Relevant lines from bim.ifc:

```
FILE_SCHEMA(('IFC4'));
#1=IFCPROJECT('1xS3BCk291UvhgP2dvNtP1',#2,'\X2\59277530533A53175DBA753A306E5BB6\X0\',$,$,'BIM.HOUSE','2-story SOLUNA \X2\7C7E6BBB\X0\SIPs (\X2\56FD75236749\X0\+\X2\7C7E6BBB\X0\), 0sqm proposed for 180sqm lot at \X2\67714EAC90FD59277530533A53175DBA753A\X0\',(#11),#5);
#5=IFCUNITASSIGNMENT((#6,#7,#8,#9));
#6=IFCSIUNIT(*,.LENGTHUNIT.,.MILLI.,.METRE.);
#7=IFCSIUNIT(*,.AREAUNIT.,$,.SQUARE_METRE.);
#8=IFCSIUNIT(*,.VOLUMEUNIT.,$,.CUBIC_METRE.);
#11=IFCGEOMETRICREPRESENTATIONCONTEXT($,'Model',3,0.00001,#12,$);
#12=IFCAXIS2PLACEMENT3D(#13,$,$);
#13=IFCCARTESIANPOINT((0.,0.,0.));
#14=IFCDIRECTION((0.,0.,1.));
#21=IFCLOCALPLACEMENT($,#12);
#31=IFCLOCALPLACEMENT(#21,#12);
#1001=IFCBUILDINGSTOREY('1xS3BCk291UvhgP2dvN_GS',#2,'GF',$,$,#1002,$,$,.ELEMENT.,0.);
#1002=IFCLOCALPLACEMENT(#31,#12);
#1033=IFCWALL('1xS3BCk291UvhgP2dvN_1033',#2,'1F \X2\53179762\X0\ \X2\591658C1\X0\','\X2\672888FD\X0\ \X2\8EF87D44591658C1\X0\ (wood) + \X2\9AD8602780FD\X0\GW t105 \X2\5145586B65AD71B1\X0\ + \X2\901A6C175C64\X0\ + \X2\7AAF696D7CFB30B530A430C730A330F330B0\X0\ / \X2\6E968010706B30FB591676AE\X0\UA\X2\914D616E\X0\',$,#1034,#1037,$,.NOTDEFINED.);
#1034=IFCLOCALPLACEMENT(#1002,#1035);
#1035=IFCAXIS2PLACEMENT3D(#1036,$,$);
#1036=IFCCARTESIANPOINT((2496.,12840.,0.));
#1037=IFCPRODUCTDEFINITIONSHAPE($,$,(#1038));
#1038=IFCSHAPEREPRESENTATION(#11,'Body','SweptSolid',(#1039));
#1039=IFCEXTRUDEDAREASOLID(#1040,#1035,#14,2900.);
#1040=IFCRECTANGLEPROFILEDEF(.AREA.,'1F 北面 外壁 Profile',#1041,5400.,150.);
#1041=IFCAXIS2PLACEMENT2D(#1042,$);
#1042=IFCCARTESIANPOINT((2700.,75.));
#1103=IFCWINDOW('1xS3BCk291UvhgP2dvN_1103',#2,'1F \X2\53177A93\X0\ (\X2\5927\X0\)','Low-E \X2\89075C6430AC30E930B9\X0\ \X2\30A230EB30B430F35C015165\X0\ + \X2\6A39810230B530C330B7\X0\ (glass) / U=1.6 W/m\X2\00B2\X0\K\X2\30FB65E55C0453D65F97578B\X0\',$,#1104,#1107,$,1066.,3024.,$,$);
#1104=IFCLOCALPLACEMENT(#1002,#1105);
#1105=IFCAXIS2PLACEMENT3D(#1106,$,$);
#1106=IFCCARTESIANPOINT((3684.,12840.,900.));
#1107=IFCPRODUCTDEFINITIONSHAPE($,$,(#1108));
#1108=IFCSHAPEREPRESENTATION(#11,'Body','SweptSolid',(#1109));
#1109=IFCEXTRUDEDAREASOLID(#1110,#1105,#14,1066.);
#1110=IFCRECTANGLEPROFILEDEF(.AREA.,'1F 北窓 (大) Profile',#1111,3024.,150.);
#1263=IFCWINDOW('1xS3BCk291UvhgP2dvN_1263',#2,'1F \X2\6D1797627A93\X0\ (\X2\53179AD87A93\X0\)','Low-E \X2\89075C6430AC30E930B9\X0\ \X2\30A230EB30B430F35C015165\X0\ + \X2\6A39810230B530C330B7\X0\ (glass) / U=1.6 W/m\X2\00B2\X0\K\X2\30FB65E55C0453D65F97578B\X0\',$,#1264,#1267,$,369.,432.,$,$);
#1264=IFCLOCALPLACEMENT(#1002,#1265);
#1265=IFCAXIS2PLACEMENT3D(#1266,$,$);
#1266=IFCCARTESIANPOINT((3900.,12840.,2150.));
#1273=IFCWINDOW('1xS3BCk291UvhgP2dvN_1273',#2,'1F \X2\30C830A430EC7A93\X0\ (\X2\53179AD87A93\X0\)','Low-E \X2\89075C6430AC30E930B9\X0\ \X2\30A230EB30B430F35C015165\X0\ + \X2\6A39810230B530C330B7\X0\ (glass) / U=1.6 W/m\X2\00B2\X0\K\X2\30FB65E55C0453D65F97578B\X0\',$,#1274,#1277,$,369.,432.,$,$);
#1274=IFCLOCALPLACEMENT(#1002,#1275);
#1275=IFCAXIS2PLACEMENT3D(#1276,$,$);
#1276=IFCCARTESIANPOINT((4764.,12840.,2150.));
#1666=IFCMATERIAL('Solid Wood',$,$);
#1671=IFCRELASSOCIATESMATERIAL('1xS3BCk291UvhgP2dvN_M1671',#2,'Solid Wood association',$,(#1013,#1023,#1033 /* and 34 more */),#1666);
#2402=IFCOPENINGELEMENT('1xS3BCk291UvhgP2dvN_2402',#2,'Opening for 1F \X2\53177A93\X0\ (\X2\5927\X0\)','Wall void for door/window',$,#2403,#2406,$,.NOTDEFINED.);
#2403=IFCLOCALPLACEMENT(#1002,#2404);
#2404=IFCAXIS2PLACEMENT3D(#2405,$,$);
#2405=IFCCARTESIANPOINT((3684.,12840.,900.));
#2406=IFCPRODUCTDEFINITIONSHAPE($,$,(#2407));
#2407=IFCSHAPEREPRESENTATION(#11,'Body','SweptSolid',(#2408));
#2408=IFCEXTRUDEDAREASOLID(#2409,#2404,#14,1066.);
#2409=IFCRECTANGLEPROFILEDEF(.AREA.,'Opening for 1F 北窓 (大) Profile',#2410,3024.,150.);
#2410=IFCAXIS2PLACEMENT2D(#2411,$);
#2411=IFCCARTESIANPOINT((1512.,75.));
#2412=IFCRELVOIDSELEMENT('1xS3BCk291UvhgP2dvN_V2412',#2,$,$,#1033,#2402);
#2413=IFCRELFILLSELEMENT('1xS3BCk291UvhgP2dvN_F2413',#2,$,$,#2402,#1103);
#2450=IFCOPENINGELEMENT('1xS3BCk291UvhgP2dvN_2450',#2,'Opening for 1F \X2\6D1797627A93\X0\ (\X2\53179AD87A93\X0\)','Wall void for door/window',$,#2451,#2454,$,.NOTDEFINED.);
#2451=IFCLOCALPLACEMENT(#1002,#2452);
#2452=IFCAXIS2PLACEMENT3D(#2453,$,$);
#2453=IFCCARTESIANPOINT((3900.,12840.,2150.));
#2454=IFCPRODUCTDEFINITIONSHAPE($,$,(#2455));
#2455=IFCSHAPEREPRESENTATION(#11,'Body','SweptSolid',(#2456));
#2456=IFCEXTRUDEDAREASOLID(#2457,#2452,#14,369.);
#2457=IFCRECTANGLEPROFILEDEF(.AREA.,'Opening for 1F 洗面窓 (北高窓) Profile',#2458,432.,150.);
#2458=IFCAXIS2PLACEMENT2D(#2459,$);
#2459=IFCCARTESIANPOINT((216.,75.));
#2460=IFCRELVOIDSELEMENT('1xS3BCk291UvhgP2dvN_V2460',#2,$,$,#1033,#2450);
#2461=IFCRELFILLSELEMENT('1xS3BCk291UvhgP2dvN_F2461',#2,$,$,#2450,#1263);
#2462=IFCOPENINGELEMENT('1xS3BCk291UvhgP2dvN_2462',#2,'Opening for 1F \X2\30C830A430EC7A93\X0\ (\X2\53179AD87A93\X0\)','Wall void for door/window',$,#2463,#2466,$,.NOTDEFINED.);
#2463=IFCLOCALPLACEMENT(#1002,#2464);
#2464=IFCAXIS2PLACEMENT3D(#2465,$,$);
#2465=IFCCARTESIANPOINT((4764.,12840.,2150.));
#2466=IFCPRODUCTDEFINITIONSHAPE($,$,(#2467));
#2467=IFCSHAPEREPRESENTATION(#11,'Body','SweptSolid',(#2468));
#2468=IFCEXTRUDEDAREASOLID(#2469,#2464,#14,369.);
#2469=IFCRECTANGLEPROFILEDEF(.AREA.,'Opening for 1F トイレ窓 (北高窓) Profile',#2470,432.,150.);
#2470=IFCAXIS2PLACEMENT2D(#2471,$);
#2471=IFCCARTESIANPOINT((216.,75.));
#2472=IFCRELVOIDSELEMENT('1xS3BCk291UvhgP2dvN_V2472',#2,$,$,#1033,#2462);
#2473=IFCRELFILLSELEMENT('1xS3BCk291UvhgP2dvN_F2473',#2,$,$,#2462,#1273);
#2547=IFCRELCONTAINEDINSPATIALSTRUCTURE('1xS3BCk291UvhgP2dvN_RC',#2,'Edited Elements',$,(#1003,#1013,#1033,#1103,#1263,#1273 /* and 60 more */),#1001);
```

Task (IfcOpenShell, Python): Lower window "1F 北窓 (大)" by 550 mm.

```python
import numpy as np
import ifcopenshell
import ifcopenshell.api.geometry
import ifcopenshell.util.placement
import ifcopenshell.util.unit

model = ifcopenshell.open("bim.ifc")
unit_scale = ifcopenshell.util.unit.calculate_unit_scale(model)

window = model.by_guid("1xS3BCk291UvhgP2dvN_1103")
opening = window.FillsVoids[0].RelatingOpeningElement
dz = -550.0

shift = np.array([0.0, 0.0, dz])
# The window is not placed relative to its opening, so move both.
for product in (opening, window):
    matrix = ifcopenshell.util.placement.get_local_placement(product.ObjectPlacement)
    matrix[:3, 3] += shift
    ifcopenshell.api.geometry.edit_object_placement(model, product=product, matrix=matrix, is_si=False)

print(f"moved by {dz * unit_scale:+.3f} m")

model.write("bim_rev.ifc")
```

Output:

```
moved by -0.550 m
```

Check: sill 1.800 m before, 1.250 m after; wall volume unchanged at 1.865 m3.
